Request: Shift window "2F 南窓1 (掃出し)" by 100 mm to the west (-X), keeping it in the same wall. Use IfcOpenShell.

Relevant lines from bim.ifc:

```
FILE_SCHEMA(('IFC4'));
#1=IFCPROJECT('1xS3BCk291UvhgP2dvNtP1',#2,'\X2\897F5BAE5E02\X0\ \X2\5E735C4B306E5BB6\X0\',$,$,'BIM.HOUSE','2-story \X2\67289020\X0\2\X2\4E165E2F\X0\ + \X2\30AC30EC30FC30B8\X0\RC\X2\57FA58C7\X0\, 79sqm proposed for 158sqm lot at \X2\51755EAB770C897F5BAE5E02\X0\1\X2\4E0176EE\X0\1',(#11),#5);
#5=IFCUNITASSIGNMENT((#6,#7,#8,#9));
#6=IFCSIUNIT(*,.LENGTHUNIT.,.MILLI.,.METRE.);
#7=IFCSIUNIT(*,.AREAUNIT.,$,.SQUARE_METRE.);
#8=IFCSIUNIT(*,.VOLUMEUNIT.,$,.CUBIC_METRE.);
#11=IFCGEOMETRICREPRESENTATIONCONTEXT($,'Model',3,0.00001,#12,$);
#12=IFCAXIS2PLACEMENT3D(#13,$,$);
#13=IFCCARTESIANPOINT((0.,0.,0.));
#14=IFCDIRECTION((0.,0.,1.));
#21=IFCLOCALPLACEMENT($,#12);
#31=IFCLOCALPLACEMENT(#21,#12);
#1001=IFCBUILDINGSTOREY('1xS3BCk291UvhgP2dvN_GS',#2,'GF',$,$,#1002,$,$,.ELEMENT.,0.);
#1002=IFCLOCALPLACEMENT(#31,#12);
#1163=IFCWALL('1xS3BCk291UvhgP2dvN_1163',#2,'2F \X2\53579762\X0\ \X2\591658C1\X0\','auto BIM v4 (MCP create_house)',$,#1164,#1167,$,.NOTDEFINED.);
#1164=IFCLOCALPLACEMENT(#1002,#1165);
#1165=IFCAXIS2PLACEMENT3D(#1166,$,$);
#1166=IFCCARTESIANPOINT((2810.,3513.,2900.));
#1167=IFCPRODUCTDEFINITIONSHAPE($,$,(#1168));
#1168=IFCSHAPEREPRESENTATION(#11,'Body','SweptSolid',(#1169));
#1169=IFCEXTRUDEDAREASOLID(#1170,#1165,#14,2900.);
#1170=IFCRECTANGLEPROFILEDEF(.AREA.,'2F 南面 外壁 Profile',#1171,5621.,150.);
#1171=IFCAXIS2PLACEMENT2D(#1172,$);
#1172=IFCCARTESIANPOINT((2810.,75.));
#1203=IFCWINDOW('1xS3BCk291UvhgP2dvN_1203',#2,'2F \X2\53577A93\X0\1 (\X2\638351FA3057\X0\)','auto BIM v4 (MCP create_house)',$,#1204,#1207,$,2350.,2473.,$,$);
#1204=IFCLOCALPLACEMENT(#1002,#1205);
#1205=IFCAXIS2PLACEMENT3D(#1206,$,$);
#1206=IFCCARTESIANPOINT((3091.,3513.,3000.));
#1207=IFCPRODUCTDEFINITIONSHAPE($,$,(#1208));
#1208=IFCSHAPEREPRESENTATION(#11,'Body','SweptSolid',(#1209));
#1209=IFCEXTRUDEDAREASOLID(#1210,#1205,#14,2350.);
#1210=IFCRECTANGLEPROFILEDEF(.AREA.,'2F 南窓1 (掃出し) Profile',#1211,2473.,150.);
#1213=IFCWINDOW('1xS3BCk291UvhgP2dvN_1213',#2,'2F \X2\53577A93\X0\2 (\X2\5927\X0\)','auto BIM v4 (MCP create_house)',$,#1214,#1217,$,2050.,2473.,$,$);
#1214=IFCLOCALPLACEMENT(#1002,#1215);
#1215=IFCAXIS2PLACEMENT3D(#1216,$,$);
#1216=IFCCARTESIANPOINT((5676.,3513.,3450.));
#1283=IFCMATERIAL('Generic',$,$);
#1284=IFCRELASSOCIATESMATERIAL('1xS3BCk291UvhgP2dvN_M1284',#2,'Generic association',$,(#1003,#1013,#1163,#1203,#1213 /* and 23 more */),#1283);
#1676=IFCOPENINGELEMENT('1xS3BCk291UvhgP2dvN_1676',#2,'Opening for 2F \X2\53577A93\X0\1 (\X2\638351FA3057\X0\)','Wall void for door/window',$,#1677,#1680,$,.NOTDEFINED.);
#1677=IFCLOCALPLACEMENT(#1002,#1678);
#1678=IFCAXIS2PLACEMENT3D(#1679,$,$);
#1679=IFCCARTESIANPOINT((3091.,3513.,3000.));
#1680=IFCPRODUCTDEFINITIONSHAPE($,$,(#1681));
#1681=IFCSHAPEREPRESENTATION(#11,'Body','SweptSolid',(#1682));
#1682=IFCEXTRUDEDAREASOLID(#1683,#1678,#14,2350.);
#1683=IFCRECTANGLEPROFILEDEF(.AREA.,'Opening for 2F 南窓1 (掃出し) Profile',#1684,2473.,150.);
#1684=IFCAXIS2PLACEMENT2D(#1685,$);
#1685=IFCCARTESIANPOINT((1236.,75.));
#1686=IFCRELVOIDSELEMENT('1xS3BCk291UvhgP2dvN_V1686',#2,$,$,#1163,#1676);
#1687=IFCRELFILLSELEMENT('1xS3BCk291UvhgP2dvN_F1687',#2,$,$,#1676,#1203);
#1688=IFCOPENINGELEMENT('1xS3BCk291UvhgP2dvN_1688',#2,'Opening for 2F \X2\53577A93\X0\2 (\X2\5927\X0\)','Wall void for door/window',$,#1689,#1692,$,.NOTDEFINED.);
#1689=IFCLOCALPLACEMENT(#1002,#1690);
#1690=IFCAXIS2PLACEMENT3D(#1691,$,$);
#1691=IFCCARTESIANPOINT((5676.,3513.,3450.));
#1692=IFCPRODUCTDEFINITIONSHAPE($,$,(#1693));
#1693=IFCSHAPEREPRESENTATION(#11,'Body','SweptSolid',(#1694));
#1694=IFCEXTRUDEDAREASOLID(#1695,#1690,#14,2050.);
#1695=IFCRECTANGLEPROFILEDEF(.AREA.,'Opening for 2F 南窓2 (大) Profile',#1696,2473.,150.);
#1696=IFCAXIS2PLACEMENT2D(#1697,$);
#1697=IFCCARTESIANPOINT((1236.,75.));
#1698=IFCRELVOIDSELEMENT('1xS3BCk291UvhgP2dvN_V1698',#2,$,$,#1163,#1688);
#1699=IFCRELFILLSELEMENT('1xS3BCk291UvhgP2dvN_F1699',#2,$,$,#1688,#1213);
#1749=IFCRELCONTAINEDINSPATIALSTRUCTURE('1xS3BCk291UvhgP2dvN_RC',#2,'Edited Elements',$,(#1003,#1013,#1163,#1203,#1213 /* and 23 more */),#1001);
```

```python
import ifcopenshell
import ifcopenshell.api.geometry
import ifcopenshell.util.placement

model = ifcopenshell.open("bim.ifc")

window = model.by_guid("1xS3BCk291UvhgP2dvN_1203")
opening = window.FillsVoids[0].RelatingOpeningElement
wall = opening.VoidsElements[0].RelatingBuildingElement

wall_matrix = ifcopenshell.util.placement.get_local_placement(wall.ObjectPlacement)
shift = wall_matrix[:3, 0] * -100.0
before = ifcopenshell.util.placement.get_local_placement(window.ObjectPlacement)[:3, 3].copy()

# The window is not placed relative to its opening, so move both.
for product in (opening, window):
    matrix = ifcopenshell.util.placement.get_local_placement(product.ObjectPlacement)
    matrix[:3, 3] += shift
    ifcopenshell.api.geometry.edit_object_placement(model, product=product, matrix=matrix, is_si=False)

after = ifcopenshell.util.placement.get_local_placement(window.ObjectPlacement)[:3, 3]
print("window moved by", (after - before).round(3) + 0.0)

model.write("bim-out.ifc")
```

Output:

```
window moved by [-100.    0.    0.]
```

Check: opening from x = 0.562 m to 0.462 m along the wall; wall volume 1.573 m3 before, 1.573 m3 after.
